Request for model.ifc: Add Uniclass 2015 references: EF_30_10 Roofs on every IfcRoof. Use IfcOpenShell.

First a look at what the model holds.

```python
import ifcopenshell

model = ifcopenshell.open("model.ifc")
print(model.schema)
print("classifications:", [c.Name for c in model.by_type("IfcClassification")])
for ifc_class in ("IfcDoor", "IfcRoof", "IfcStair", "IfcWall", "IfcWindow"):
    print(ifc_class, len(model.by_type(ifc_class)))
```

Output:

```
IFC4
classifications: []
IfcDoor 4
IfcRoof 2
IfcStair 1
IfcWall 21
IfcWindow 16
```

```python
import ifcopenshell
import ifcopenshell.api.classification

model = ifcopenshell.open("model.ifc")

system = ifcopenshell.api.classification.add_classification(model, classification="Uniclass 2015")

codes = {
    "IfcRoof": ("EF_30_10", "Roofs"),
}
for ifc_class, (code, name) in codes.items():
    products = model.by_type(ifc_class)
    ifcopenshell.api.classification.add_reference(
        model, products=products, classification=system, identification=code, name=name
    )
    print(code, len(products))

model.write("model_rev.ifc")
```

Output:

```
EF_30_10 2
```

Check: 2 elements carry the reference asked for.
